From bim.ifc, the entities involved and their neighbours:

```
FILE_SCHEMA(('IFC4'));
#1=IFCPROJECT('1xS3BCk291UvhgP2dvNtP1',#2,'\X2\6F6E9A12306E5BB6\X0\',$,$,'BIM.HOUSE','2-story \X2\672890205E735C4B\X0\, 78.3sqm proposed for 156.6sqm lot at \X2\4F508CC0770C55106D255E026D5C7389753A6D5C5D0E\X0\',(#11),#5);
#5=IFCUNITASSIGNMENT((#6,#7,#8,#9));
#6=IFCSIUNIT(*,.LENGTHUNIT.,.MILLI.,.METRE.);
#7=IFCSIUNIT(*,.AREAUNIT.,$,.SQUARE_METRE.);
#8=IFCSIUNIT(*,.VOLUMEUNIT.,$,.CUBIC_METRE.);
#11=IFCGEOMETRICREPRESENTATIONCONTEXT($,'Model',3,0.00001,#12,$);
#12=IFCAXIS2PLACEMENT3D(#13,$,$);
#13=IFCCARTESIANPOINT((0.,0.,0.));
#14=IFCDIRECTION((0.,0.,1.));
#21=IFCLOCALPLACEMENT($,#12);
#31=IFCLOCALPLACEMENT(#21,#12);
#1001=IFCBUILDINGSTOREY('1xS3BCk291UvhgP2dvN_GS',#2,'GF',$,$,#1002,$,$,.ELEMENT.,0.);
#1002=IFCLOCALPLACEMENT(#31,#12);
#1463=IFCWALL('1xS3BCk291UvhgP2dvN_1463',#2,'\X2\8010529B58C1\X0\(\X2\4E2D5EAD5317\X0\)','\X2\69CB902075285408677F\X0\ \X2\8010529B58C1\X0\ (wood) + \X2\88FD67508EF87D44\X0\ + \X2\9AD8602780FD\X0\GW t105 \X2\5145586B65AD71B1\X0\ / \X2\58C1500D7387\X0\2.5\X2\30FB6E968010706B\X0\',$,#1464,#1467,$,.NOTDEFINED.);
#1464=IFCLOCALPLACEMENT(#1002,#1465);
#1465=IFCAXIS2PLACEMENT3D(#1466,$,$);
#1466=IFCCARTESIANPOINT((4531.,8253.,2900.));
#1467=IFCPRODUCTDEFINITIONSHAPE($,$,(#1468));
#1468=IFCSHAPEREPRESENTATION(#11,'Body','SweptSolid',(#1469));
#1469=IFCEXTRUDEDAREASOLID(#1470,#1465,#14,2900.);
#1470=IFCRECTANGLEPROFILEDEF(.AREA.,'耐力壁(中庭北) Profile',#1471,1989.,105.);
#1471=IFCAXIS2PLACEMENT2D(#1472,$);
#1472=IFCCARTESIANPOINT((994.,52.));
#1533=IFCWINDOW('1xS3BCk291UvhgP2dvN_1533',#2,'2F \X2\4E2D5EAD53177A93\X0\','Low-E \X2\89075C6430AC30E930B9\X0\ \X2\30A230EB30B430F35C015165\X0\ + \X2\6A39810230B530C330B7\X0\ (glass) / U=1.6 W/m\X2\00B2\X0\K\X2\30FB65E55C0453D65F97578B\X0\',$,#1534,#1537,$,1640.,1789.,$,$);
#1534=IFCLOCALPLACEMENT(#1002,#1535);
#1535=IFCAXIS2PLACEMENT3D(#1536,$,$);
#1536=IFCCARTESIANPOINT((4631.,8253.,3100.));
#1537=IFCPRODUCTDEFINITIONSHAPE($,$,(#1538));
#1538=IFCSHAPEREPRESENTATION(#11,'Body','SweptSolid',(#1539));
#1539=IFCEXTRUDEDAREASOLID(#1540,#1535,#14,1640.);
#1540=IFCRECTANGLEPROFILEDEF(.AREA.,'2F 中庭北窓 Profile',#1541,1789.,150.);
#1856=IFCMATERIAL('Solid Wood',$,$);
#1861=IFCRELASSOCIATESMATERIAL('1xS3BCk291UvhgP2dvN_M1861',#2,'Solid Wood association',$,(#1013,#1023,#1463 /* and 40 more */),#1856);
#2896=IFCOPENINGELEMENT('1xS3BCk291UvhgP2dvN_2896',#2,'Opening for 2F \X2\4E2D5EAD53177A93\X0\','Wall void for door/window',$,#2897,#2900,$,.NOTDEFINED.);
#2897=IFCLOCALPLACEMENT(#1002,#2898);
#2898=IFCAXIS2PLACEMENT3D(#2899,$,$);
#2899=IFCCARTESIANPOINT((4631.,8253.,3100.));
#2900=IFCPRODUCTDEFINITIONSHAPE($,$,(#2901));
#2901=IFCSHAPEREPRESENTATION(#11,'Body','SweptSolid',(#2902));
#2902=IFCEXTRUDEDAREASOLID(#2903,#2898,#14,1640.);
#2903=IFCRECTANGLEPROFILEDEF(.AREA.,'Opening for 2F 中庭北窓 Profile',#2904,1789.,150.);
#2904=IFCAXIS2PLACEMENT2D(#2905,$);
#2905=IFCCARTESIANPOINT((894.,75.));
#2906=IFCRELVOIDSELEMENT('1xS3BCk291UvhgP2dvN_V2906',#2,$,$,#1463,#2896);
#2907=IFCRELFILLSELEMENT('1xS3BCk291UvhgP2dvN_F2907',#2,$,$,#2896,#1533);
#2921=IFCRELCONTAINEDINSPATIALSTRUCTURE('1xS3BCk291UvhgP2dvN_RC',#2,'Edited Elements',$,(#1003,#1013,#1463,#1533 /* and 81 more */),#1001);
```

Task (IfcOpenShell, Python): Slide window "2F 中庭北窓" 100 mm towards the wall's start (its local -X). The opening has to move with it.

```python
import ifcopenshell
import ifcopenshell.api.geometry
import ifcopenshell.util.placement
import ifcopenshell.util.unit

model = ifcopenshell.open("bim.ifc")
unit_scale = ifcopenshell.util.unit.calculate_unit_scale(model)

window = model.by_id(1533)
opening = window.FillsVoids[0].RelatingOpeningElement
wall = opening.VoidsElements[0].RelatingBuildingElement

wall_matrix = ifcopenshell.util.placement.get_local_placement(wall.ObjectPlacement)
shift = wall_matrix[:3, 0] * -0.1 / unit_scale
before = ifcopenshell.util.placement.get_local_placement(window.ObjectPlacement)[:3, 3].copy()

# The window is not placed relative to its opening, so move both.
for product in (opening, window):
    matrix = ifcopenshell.util.placement.get_local_placement(product.ObjectPlacement)
    matrix[:3, 3] += shift
    ifcopenshell.api.geometry.edit_object_placement(model, product=product, matrix=matrix, is_si=False)

after = ifcopenshell.util.placement.get_local_placement(window.ObjectPlacement)[:3, 3]
print("window moved by", (after - before).round(3) + 0.0)

model.write("bim-out.ifc")
```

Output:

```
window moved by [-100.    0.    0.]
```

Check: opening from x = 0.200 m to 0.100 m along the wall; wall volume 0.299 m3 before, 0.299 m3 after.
